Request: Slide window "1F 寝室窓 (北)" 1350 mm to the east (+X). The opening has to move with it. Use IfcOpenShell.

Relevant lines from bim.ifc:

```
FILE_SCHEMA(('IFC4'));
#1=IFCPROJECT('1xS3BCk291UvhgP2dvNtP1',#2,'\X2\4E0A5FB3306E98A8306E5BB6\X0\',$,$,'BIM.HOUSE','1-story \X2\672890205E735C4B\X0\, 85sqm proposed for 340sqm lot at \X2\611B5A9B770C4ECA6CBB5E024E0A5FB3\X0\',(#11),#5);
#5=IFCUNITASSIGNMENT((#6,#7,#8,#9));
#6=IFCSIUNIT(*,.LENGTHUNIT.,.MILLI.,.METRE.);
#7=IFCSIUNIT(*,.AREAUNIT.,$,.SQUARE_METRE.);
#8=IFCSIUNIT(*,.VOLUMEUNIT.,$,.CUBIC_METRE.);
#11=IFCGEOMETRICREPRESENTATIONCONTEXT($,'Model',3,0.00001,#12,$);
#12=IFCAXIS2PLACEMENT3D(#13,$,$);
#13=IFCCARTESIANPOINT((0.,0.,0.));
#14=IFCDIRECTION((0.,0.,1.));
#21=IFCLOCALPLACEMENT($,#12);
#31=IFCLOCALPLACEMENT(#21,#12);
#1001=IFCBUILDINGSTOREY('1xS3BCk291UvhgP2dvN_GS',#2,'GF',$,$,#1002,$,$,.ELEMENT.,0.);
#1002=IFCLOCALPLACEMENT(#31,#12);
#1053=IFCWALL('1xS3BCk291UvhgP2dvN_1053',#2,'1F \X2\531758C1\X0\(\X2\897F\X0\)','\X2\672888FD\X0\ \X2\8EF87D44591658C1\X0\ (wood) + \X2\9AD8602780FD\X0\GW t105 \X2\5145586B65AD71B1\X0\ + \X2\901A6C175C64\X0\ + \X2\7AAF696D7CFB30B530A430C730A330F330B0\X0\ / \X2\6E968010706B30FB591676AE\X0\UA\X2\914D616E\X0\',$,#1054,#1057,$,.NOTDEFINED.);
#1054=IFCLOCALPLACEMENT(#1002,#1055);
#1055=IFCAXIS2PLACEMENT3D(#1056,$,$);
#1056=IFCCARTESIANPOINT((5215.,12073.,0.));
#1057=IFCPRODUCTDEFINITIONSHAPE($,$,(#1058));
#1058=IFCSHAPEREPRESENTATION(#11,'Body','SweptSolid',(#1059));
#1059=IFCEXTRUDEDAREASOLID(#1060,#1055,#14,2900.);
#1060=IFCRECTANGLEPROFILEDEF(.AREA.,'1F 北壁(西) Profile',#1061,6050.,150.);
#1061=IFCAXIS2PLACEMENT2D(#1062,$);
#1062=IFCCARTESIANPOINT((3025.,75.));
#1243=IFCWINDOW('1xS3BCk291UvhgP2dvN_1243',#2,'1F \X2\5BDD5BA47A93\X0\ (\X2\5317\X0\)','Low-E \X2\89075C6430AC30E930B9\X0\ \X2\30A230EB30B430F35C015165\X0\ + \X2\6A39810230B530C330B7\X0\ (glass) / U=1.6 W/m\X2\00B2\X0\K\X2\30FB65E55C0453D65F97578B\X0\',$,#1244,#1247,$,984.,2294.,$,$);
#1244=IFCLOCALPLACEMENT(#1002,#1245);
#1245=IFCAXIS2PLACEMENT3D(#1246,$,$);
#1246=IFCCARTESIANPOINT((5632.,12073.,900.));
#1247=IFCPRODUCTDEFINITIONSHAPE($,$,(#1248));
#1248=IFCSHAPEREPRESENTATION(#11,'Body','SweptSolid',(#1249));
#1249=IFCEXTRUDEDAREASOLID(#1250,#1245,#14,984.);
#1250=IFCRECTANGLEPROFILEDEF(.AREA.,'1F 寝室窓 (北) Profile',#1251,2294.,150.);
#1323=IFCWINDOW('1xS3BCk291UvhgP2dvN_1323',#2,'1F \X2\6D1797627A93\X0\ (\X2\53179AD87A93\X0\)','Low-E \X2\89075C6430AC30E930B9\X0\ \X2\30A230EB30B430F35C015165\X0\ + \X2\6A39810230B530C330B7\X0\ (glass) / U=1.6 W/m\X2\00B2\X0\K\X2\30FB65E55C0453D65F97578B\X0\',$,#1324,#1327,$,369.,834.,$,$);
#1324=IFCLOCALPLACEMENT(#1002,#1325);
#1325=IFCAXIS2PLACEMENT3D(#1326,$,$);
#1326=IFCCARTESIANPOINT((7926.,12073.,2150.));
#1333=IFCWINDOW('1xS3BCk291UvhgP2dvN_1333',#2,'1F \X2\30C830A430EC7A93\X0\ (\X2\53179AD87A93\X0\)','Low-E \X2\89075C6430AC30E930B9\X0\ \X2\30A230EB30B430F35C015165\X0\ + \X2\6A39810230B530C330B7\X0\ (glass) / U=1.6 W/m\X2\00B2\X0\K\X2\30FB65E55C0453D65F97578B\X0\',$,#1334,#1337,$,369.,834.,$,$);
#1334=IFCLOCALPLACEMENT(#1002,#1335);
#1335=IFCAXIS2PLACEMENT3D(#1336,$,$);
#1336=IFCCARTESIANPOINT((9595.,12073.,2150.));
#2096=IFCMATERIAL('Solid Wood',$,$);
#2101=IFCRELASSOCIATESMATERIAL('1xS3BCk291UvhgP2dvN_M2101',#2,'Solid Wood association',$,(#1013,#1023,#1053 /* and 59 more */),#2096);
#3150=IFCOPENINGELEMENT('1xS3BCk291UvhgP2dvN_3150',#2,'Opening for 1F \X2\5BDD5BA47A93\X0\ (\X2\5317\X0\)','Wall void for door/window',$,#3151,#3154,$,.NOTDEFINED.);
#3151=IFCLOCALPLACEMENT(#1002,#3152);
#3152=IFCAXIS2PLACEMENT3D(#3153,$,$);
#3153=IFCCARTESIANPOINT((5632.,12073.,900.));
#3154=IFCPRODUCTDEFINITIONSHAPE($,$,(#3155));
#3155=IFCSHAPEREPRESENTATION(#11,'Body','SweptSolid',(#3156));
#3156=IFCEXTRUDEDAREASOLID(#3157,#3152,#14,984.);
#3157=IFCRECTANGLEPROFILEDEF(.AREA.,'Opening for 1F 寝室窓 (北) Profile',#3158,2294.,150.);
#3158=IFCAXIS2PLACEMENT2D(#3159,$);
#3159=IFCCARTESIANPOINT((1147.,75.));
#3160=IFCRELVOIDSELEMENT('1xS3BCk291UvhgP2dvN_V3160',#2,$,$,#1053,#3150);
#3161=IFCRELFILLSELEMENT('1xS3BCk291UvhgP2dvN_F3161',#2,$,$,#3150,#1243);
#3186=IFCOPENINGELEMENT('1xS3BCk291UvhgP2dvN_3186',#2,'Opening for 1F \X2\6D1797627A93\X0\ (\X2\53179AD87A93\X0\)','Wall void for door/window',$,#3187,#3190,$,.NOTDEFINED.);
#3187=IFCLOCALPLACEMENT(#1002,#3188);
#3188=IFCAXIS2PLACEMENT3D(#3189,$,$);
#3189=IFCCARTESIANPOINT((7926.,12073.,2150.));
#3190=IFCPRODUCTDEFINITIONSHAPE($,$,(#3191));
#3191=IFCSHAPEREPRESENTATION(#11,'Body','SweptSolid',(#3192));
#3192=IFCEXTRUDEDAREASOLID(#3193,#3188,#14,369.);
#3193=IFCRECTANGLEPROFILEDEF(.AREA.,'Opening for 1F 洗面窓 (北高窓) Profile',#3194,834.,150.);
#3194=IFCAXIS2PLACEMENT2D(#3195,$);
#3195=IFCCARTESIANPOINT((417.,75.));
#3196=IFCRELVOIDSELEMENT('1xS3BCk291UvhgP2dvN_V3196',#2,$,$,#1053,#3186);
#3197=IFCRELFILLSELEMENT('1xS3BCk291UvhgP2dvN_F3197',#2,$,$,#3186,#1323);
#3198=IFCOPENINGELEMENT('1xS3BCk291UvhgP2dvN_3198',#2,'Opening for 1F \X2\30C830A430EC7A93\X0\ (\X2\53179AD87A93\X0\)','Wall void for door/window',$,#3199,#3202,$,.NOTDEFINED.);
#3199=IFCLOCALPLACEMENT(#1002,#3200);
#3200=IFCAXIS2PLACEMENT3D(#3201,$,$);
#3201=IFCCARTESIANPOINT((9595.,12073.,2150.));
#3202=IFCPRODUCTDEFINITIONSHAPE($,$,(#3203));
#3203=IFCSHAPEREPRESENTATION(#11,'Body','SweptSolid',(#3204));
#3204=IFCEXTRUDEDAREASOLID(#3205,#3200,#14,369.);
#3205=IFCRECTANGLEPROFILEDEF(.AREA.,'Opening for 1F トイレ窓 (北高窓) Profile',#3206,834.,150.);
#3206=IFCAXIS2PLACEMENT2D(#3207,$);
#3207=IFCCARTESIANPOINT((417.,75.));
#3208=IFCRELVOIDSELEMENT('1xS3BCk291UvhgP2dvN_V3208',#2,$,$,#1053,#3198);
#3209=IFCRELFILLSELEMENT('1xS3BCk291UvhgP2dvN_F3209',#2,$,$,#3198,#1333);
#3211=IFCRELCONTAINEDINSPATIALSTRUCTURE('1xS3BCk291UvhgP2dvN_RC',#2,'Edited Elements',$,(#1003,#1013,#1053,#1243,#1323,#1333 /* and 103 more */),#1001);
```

```python
import ifcopenshell
import ifcopenshell.api.geometry
import ifcopenshell.util.placement
import ifcopenshell.util.unit

model = ifcopenshell.open("bim.ifc")
unit_scale = ifcopenshell.util.unit.calculate_unit_scale(model)

window = model.by_guid("1xS3BCk291UvhgP2dvN_1243")
opening = window.FillsVoids[0].RelatingOpeningElement
wall = opening.VoidsElements[0].RelatingBuildingElement

wall_matrix = ifcopenshell.util.placement.get_local_placement(wall.ObjectPlacement)
shift = wall_matrix[:3, 0] * 1.35 / unit_scale
before = ifcopenshell.util.placement.get_local_placement(window.ObjectPlacement)[:3, 3].copy()

# The window is not placed relative to its opening, so move both.
for product in (opening, window):
    matrix = ifcopenshell.util.placement.get_local_placement(product.ObjectPlacement)
    matrix[:3, 3] += shift
    ifcopenshell.api.geometry.edit_object_placement(model, product=product, matrix=matrix, is_si=False)

after = ifcopenshell.util.placement.get_local_placement(window.ObjectPlacement)[:3, 3]
print("window moved by", (after - before).round(3) + 0.0)

model.write("bim-out.ifc")
```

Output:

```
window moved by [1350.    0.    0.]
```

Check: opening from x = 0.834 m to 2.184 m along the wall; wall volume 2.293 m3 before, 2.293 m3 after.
